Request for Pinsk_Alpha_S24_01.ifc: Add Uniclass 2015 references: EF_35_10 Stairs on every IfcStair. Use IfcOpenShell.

First a look at what the model holds.

```python
import ifcopenshell

model = ifcopenshell.open("Pinsk_Alpha_S24_01.ifc")
print(model.schema)
print("classifications:", [c.Name for c in model.by_type("IfcClassification")])
for ifc_class in ("IfcDoor", "IfcRoof", "IfcStair", "IfcWall", "IfcWindow"):
    print(ifc_class, len(model.by_type(ifc_class)))
```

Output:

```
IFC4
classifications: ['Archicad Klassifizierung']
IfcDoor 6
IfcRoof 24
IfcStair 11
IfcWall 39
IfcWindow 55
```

```python
import ifcopenshell
import ifcopenshell.api.classification

model = ifcopenshell.open("Pinsk_Alpha_S24_01.ifc")

system = ifcopenshell.api.classification.add_classification(model, classification="Uniclass 2015")

codes = {
    "IfcStair": ("EF_35_10", "Stairs"),
}
for ifc_class, (code, name) in codes.items():
    products = model.by_type(ifc_class)
    ifcopenshell.api.classification.add_reference(
        model, products=products, classification=system, identification=code, name=name
    )
    print(code, len(products))

model.write("Pinsk_Alpha_S24_01_updated.ifc")
```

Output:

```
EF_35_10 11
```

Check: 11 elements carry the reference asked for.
